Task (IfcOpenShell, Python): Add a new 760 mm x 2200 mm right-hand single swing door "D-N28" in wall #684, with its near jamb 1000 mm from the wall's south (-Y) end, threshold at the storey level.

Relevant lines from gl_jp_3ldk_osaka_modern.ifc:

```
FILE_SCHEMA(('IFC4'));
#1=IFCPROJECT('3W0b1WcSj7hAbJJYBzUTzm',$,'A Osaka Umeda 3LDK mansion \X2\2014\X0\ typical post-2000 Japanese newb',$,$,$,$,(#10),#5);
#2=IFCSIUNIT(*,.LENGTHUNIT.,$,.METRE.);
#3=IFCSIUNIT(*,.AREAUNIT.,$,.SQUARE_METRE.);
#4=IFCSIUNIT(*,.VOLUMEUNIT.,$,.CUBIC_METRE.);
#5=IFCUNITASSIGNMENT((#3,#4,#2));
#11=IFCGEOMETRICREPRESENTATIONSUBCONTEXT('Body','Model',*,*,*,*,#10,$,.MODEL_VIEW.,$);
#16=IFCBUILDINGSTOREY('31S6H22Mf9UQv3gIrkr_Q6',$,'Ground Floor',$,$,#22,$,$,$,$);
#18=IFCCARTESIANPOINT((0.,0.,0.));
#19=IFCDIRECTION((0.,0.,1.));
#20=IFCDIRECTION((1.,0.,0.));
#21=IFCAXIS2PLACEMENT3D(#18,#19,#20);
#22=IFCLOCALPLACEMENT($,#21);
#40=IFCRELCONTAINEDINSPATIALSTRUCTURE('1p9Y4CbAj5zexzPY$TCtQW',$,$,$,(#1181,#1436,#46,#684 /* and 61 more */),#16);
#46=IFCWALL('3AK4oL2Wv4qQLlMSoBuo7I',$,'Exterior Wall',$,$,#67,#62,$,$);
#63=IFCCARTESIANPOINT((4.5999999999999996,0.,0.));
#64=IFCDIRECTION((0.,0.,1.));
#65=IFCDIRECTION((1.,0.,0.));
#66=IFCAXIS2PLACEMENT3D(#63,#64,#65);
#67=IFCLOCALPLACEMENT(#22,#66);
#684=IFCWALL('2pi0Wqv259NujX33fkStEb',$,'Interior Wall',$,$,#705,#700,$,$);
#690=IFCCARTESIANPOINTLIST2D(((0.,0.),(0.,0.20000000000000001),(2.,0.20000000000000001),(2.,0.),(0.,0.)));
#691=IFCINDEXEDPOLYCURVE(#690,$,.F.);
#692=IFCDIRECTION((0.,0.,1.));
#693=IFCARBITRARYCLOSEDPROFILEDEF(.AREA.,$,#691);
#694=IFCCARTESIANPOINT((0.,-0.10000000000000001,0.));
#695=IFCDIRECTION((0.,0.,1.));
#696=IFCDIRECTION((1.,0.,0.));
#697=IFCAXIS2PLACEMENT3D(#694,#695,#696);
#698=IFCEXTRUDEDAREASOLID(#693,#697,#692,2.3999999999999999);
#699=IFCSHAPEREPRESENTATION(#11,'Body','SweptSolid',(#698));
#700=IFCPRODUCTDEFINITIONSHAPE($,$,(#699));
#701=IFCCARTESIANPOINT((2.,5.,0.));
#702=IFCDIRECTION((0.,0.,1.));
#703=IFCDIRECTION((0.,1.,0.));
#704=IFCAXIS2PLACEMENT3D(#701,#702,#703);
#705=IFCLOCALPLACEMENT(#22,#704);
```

```python
import numpy as np
import ifcopenshell
import ifcopenshell.api.feature
import ifcopenshell.api.geometry
import ifcopenshell.api.root
import ifcopenshell.api.spatial
import ifcopenshell.geom
import ifcopenshell.util.element
import ifcopenshell.util.placement
import ifcopenshell.util.representation
import ifcopenshell.util.shape
import ifcopenshell.util.unit

model = ifcopenshell.open("gl_jp_3ldk_osaka_modern.ifc")
unit_scale = ifcopenshell.util.unit.calculate_unit_scale(model)
settings = ifcopenshell.geom.settings()


def volume(element):
    """Net volume in cubic metres, openings subtracted."""
    shape = ifcopenshell.geom.create_shape(settings, element)
    return ifcopenshell.util.shape.get_volume(shape.geometry)


wall = model.by_guid("2pi0Wqv259NujX33fkStEb")
storey = ifcopenshell.util.element.get_container(wall, ifc_class="IfcBuildingStorey")
context = ifcopenshell.util.representation.get_context(model, "Model", "Body", "MODEL_VIEW")
before = volume(wall)

width, height, from_end, sill = 0.76, 2.2, 1, 0.0  # metres

# The wall runs along its own X axis, and the end named is its -X end.
wall_shape = ifcopenshell.geom.create_shape(settings, wall)
x, y, z = ifcopenshell.util.shape.get_vertices(wall_shape.geometry).T
start = x.min() + from_end
face, thickness = float(y.min()), float(y.max() - y.min())
wall_matrix = ifcopenshell.util.placement.get_local_placement(wall.ObjectPlacement)
level = ifcopenshell.util.placement.get_local_placement(storey.ObjectPlacement)[2, 3]


def in_wall(x, y):
    """Placement at x, y metres in the wall's axes, at sill height."""
    matrix = wall_matrix.copy()
    matrix[:, 3] = wall_matrix @ np.array([x / unit_scale, y / unit_scale, 0.0, 1.0])
    matrix[2, 3] = level + sill / unit_scale
    return matrix


# Opening: a box that overshoots both wall faces by 50 mm.
opening = ifcopenshell.api.root.create_entity(model, ifc_class="IfcOpeningElement", predefined_type="OPENING")
box = ifcopenshell.api.geometry.add_wall_representation(
    model, context=context, length=width, height=height, thickness=thickness + 0.1
)
ifcopenshell.api.geometry.assign_representation(model, product=opening, representation=box)
ifcopenshell.api.geometry.edit_object_placement(model, product=opening, matrix=in_wall(start, face - 0.05), is_si=False)
ifcopenshell.api.feature.add_feature(model, feature=opening, element=wall)

door = ifcopenshell.api.root.create_entity(model, ifc_class="IfcDoor", name="D-N28", predefined_type="DOOR")
door.OverallWidth, door.OverallHeight = width / unit_scale, height / unit_scale
door.OperationType = "SINGLE_SWING_RIGHT"
body = ifcopenshell.api.geometry.add_door_representation(
    model,
    context=context,
    overall_width=door.OverallWidth,
    overall_height=door.OverallHeight,
    operation_type="SINGLE_SWING_RIGHT",
    lining_properties={"LiningDepth": thickness / unit_scale, "ThresholdDepth": thickness / unit_scale},
)
ifcopenshell.api.geometry.assign_representation(model, product=door, representation=body)
ifcopenshell.api.spatial.assign_container(model, products=[door], relating_structure=storey)
ifcopenshell.api.feature.add_filling(model, opening=opening, element=door)

# The lining spans the wall, so the door starts at the wall face.
ifcopenshell.api.geometry.edit_object_placement(model, product=door, matrix=in_wall(start, face), is_si=False)

after = volume(wall)

print(f"wall volume {before:.3f} -> {after:.3f} m3")

model.write("gl_jp_3ldk_osaka_modern_edited.ifc")
```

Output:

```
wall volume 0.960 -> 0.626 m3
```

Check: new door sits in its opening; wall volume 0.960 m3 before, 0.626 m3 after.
